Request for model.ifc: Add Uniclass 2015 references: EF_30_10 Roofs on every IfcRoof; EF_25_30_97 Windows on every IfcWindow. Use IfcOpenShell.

First a look at what the model holds.

```python
import ifcopenshell

model = ifcopenshell.open("model.ifc")
print(model.schema)
print("classifications:", [c.Name for c in model.by_type("IfcClassification")])
for ifc_class in ("IfcDoor", "IfcRoof", "IfcStair", "IfcWall", "IfcWindow"):
    print(ifc_class, len(model.by_type(ifc_class)))
```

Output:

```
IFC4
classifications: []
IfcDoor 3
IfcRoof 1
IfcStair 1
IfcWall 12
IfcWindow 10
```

```python
import ifcopenshell
import ifcopenshell.api.classification

model = ifcopenshell.open("model.ifc")

system = ifcopenshell.api.classification.add_classification(model, classification="Uniclass 2015")

codes = {
    "IfcRoof": ("EF_30_10", "Roofs"),
    "IfcWindow": ("EF_25_30_97", "Windows"),
}
for ifc_class, (code, name) in codes.items():
    products = model.by_type(ifc_class)
    ifcopenshell.api.classification.add_reference(
        model, products=products, classification=system, identification=code, name=name
    )
    print(code, len(products))

model.write("model_edited.ifc")
```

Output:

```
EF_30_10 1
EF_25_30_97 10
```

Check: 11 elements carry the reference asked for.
